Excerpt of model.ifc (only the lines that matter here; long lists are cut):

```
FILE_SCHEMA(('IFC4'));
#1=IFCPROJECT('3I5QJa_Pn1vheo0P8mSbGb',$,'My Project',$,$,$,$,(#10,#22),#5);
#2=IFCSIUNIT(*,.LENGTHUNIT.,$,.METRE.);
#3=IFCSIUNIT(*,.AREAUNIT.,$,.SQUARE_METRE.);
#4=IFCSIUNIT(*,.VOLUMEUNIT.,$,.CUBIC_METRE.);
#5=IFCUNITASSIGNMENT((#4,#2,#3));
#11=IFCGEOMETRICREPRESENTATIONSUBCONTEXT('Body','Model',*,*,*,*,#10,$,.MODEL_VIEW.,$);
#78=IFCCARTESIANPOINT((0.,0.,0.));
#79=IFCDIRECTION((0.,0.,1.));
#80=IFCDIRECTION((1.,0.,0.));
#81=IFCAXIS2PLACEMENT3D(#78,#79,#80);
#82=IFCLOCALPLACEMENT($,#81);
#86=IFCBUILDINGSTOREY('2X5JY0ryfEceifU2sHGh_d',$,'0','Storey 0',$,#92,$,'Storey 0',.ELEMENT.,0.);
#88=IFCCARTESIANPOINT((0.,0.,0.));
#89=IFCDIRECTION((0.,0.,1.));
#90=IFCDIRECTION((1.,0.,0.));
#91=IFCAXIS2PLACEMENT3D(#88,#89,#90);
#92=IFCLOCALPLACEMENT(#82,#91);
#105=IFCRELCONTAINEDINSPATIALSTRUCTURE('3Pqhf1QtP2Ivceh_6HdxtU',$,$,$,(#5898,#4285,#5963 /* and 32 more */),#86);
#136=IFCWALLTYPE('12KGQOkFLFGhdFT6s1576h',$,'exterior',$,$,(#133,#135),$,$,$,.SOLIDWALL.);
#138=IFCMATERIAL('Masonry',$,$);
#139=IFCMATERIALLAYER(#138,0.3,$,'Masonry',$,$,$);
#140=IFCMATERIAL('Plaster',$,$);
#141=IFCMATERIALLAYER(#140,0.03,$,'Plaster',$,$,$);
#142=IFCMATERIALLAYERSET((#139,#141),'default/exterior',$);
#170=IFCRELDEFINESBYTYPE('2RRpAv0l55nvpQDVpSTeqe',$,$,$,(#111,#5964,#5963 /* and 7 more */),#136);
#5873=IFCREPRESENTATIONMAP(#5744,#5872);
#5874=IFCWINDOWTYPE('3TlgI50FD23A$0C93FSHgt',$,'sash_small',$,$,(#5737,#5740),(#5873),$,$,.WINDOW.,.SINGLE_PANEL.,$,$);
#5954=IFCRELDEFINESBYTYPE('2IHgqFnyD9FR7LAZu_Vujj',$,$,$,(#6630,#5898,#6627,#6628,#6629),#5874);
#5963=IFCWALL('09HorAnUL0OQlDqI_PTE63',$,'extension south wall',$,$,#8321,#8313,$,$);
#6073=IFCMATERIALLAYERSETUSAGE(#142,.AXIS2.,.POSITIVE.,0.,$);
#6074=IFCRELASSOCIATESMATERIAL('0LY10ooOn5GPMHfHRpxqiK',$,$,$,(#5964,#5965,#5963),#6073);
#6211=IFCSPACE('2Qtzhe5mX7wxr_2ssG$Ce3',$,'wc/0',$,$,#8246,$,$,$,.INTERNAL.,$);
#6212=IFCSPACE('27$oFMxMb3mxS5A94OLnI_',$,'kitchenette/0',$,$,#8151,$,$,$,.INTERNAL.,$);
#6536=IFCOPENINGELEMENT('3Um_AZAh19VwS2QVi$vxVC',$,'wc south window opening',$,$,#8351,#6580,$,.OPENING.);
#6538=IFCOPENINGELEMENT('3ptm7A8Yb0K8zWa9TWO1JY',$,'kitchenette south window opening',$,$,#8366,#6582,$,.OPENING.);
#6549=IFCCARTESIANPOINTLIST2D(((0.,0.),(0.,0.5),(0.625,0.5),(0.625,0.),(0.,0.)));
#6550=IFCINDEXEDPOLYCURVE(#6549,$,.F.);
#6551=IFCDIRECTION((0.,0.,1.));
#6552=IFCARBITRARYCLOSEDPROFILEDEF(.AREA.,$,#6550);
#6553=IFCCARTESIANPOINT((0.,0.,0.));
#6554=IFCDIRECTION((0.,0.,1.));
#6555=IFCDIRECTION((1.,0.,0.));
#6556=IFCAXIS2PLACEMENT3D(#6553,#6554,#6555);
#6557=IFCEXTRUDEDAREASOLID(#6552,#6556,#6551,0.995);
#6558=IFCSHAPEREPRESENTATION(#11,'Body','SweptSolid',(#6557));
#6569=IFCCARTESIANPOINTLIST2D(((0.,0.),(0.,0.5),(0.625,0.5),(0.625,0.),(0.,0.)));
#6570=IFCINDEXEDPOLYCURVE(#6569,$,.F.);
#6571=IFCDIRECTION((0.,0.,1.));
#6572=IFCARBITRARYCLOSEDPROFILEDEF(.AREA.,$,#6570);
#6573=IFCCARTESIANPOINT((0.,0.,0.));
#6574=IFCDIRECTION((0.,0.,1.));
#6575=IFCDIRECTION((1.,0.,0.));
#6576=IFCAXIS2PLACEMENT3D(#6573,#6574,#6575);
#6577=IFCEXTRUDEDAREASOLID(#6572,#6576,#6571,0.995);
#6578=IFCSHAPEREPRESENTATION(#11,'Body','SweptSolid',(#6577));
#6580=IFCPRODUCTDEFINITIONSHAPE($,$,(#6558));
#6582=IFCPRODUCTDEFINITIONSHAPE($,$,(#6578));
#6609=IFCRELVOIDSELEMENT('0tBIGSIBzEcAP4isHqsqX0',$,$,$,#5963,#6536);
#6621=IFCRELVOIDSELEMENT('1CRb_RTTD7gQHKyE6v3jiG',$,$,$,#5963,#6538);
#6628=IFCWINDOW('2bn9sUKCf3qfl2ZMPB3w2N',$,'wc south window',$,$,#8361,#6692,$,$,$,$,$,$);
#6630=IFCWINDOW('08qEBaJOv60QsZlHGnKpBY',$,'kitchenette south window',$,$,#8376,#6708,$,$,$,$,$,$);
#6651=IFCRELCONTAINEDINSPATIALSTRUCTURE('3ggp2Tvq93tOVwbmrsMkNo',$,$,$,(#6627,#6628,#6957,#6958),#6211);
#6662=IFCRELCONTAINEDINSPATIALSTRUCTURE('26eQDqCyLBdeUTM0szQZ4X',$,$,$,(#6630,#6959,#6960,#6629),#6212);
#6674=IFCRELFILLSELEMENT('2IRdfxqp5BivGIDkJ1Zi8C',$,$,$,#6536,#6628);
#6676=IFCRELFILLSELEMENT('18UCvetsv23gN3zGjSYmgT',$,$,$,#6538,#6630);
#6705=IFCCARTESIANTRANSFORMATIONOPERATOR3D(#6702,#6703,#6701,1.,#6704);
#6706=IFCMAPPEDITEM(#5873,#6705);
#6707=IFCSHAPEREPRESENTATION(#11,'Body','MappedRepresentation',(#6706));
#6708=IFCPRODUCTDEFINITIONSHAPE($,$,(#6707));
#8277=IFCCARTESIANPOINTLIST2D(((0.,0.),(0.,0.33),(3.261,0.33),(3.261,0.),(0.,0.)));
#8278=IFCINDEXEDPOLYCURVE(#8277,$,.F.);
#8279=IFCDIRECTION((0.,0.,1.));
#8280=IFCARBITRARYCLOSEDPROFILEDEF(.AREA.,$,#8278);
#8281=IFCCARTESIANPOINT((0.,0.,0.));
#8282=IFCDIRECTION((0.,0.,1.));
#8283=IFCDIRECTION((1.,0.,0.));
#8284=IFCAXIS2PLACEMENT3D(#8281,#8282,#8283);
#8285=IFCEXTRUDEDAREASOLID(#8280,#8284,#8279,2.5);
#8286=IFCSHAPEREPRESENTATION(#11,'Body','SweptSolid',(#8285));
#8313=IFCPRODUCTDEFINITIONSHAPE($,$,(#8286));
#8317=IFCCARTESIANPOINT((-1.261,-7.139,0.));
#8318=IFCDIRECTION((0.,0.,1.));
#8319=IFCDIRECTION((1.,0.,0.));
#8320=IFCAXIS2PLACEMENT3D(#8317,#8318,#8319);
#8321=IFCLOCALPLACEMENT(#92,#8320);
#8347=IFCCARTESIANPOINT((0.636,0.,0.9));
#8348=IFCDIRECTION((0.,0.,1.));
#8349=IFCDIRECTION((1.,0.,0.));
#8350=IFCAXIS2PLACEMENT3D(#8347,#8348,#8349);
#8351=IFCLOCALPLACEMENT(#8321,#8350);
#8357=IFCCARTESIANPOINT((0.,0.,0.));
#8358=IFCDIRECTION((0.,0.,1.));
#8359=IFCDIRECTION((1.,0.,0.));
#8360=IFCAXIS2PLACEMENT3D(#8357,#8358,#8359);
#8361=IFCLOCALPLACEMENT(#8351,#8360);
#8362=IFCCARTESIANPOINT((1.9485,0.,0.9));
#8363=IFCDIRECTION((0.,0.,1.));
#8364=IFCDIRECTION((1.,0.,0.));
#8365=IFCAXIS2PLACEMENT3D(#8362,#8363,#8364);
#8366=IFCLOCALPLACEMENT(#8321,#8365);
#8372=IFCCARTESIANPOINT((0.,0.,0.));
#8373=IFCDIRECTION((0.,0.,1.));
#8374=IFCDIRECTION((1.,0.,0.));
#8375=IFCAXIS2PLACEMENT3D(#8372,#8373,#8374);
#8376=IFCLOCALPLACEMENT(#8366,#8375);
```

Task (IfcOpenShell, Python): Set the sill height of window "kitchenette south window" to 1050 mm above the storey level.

```python
import numpy as np
import ifcopenshell
import ifcopenshell.api.geometry
import ifcopenshell.geom
import ifcopenshell.util.element
import ifcopenshell.util.placement
import ifcopenshell.util.shape
import ifcopenshell.util.unit

model = ifcopenshell.open("model.ifc")
unit_scale = ifcopenshell.util.unit.calculate_unit_scale(model)

window = model.by_guid("08qEBaJOv60QsZlHGnKpBY")
opening = window.FillsVoids[0].RelatingOpeningElement
storey = ifcopenshell.util.element.get_container(window, ifc_class="IfcBuildingStorey")
level = ifcopenshell.util.placement.get_local_placement(storey.ObjectPlacement)[2, 3]

# The opening's origin need not be at the sill, so measure its lowest point.
shape = ifcopenshell.geom.create_shape(ifcopenshell.geom.settings(), opening)
bottom = ifcopenshell.util.shape.get_shape_bottom_elevation(shape, shape.geometry) / unit_scale
dz = level + 1.05 - bottom

shift = np.array([0.0, 0.0, dz])
# The window is placed relative to its opening, so it follows when the opening moves.
matrix = ifcopenshell.util.placement.get_local_placement(opening.ObjectPlacement)
matrix[:3, 3] += shift
ifcopenshell.api.geometry.edit_object_placement(
    model, product=opening, matrix=matrix, is_si=False, should_transform_children=True
)

print(f"moved by {dz * unit_scale:+.3f} m")

model.write("model_v2.ifc")
```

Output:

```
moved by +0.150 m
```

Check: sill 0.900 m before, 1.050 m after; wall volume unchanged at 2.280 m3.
